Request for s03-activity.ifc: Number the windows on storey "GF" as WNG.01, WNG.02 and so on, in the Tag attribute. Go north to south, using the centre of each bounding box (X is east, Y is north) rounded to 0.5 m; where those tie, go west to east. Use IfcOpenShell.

First a look at what the model holds.

```python
import ifcopenshell
import ifcopenshell.util.element
import ifcopenshell.util.placement

model = ifcopenshell.open("s03-activity.ifc")
print(model.schema)
storey = next(s for s in model.by_type("IfcBuildingStorey") if s.Name == "GF")
windows = [e for e in ifcopenshell.util.element.get_decomposition(storey) if e.is_a("IfcWindow")]
for e in sorted(windows, key=lambda e: e.id()):
    origin = ifcopenshell.util.placement.get_local_placement(e.ObjectPlacement)[:3, 3]
    print(e.id(), e.Tag, e.Name, origin.round(2) + 0.0, sep=" | ")
```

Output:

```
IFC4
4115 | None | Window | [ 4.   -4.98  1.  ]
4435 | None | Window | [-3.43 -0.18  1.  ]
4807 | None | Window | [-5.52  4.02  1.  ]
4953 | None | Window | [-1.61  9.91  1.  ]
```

```python
import ifcopenshell
import ifcopenshell.geom
import ifcopenshell.util.element
import ifcopenshell.util.shape

model = ifcopenshell.open("s03-activity.ifc")
settings = ifcopenshell.geom.settings()
settings.set("use-world-coords", True)


def centre(element):
    shape = ifcopenshell.geom.create_shape(settings, element)
    return ifcopenshell.util.shape.get_bbox_centroid(shape.geometry)


storey = next(s for s in model.by_type("IfcBuildingStorey") if s.Name == "GF")
windows = [e for e in ifcopenshell.util.element.get_decomposition(storey) if e.is_a("IfcWindow")]

# Insertion points can sit at a corner or the storey origin, so sort by the geometry (in metres).
centres = {e: centre(e) for e in windows}
windows.sort(key=lambda e: (-round(centres[e][1] / 0.5), centres[e][0]))

for i, e in enumerate(windows, start=1):
    number = f"WNG.{i:02d}"
    e.Tag = number
    print(e.id(), number)

model.write("s03-activity_v2.ifc")
```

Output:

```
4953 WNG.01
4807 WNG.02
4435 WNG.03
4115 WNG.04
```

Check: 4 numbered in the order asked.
